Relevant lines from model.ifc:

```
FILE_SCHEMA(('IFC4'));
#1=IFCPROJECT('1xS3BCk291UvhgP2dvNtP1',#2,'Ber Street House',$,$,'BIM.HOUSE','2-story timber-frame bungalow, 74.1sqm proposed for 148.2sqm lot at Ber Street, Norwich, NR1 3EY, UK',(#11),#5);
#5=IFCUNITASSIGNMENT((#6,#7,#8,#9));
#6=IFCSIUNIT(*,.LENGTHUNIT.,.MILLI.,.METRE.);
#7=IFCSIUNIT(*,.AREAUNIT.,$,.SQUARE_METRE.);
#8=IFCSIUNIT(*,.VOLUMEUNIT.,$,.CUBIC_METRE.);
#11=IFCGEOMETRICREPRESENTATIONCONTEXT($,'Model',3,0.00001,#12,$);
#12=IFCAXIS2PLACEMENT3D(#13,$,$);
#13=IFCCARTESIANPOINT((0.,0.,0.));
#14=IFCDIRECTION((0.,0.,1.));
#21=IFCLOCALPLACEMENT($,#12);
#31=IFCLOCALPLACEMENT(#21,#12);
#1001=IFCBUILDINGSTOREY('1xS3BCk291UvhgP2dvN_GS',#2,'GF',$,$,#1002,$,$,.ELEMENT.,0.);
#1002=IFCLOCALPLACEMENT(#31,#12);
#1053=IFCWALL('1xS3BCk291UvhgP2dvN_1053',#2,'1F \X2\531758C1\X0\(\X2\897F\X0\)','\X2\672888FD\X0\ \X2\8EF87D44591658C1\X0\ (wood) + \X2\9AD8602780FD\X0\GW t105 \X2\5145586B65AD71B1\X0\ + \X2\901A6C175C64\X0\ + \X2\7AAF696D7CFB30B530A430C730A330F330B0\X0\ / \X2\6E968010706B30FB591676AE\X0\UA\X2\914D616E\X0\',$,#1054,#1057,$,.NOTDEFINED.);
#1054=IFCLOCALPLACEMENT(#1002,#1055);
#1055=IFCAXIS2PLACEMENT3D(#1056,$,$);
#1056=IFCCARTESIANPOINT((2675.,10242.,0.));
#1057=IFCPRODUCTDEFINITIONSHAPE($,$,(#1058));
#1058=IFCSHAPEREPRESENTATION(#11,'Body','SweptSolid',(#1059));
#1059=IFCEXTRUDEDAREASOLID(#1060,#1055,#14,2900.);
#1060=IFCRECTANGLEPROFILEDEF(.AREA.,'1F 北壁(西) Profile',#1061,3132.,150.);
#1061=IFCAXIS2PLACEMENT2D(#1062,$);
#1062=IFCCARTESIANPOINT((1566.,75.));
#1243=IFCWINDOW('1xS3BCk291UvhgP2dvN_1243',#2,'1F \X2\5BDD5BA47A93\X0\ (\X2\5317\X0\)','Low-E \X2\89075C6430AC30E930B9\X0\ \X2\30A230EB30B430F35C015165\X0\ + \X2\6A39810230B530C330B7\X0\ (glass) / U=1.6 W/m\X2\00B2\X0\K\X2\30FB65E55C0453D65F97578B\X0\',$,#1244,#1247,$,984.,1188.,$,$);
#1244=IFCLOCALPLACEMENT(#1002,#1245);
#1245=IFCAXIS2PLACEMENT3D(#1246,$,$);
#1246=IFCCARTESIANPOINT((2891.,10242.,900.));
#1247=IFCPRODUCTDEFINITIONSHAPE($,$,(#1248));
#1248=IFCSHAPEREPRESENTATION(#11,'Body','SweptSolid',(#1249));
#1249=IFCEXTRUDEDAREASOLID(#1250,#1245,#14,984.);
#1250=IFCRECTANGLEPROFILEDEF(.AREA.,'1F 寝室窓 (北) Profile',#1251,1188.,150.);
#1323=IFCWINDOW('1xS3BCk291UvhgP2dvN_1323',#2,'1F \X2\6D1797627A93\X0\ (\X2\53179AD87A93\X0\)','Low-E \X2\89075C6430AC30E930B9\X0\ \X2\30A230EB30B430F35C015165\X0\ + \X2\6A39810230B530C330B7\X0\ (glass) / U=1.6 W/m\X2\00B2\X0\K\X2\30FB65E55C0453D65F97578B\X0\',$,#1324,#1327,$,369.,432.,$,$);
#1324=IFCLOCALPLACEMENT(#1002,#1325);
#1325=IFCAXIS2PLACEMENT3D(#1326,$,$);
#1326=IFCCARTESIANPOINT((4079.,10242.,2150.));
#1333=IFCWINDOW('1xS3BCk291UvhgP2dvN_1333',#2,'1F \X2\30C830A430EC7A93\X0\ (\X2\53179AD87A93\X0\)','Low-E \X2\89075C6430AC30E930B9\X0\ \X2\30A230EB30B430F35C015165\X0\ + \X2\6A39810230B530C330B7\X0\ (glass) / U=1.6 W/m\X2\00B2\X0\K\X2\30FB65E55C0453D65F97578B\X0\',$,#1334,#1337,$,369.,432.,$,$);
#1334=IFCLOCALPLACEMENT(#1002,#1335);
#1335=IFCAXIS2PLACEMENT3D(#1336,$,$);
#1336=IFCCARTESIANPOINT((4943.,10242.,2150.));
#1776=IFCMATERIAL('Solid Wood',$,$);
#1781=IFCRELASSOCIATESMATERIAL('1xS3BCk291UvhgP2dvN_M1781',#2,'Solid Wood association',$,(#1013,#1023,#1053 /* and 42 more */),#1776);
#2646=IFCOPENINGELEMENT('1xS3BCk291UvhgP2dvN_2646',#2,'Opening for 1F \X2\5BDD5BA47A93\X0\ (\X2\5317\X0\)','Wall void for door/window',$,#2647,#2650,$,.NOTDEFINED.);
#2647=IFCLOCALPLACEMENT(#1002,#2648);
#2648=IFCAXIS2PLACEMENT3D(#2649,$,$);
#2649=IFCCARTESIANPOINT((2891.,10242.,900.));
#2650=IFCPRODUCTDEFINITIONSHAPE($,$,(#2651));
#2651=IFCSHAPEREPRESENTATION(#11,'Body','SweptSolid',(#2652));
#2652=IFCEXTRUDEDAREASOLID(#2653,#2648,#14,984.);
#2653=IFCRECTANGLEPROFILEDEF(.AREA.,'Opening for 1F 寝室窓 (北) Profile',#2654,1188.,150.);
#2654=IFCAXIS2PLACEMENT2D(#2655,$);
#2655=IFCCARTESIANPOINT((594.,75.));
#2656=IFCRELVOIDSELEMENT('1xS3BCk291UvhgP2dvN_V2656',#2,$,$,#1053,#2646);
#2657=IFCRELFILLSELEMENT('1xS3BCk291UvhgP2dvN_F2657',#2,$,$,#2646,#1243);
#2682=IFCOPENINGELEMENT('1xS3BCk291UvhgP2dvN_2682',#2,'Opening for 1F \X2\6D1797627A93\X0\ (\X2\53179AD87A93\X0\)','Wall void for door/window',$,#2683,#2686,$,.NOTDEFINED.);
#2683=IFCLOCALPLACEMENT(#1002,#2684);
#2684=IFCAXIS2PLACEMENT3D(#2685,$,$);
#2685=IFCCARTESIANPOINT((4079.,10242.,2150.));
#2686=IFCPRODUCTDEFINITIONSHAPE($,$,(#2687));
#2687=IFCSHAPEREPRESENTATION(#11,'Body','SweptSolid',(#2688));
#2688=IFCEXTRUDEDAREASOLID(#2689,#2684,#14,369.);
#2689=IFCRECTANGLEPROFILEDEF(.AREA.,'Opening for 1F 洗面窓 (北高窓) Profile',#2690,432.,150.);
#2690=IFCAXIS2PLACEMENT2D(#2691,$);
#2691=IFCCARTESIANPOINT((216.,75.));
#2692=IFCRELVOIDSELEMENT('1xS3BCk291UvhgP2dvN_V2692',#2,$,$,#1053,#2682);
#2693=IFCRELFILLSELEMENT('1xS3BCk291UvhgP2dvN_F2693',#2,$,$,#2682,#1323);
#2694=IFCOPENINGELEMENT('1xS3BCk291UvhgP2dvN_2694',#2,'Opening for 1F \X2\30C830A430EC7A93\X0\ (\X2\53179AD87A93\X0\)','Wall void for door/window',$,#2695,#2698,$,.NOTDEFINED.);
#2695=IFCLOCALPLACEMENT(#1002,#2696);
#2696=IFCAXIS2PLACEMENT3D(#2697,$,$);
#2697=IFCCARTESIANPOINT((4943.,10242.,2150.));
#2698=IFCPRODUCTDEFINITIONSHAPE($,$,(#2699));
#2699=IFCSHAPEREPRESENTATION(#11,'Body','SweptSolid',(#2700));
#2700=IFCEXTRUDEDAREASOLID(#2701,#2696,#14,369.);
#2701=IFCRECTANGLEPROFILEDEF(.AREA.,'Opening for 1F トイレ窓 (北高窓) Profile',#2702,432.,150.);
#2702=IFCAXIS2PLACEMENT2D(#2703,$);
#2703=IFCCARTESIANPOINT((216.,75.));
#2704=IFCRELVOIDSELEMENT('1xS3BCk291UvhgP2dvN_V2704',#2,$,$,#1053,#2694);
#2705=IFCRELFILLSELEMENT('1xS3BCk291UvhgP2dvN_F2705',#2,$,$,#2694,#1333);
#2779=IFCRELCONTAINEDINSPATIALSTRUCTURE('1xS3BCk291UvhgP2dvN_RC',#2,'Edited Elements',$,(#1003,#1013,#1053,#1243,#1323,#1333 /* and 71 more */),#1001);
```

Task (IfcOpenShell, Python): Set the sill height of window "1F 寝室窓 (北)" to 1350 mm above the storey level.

```python
import numpy as np
import ifcopenshell
import ifcopenshell.api.geometry
import ifcopenshell.geom
import ifcopenshell.util.element
import ifcopenshell.util.placement
import ifcopenshell.util.shape
import ifcopenshell.util.unit

model = ifcopenshell.open("model.ifc")
unit_scale = ifcopenshell.util.unit.calculate_unit_scale(model)

window = model.by_id(1243)
opening = window.FillsVoids[0].RelatingOpeningElement
storey = ifcopenshell.util.element.get_container(window, ifc_class="IfcBuildingStorey")
level = ifcopenshell.util.placement.get_local_placement(storey.ObjectPlacement)[2, 3]

# The opening's origin need not be at the sill, so measure its lowest point.
shape = ifcopenshell.geom.create_shape(ifcopenshell.geom.settings(), opening)
bottom = ifcopenshell.util.shape.get_shape_bottom_elevation(shape, shape.geometry) / unit_scale
dz = level + 1350.0 - bottom

shift = np.array([0.0, 0.0, dz])
# The window is not placed relative to its opening, so move both.
for product in (opening, window):
    matrix = ifcopenshell.util.placement.get_local_placement(product.ObjectPlacement)
    matrix[:3, 3] += shift
    ifcopenshell.api.geometry.edit_object_placement(model, product=product, matrix=matrix, is_si=False)

print(f"moved by {dz * unit_scale:+.3f} m")

model.write("model-out.ifc")
```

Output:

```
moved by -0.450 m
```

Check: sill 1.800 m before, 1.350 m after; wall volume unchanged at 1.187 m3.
